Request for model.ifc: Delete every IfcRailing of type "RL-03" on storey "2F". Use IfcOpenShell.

First a look at what the model holds.

```python
import ifcopenshell
import ifcopenshell.util.element

model = ifcopenshell.open("model.ifc")
print(model.schema)
storey = next(s for s in model.by_type("IfcBuildingStorey") if s.Name == "2F")
railings = [e for e in ifcopenshell.util.element.get_decomposition(storey) if e.is_a("IfcRailing")]
seen = {}
for e in railings:
    element_type = ifcopenshell.util.element.get_type(e)
    name = element_type.Name if element_type not in (None, e) else None
    seen[name] = seen.get(name, 0) + 1
for name, count in sorted(seen.items(), key=str):
    print(count, "x", name)
```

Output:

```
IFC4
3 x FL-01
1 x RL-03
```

```python
import ifcopenshell
import ifcopenshell.api.root
import ifcopenshell.util.element

model = ifcopenshell.open("model.ifc")

storey = next(s for s in model.by_type("IfcBuildingStorey") if s.Name == "2F")
railings = [e for e in ifcopenshell.util.element.get_decomposition(storey) if e.is_a("IfcRailing")]
targets = [e for e in railings if (t := ifcopenshell.util.element.get_type(e)) not in (None, e) and t.Name == "RL-03"]

for e in targets:
    ifcopenshell.api.root.remove_product(model, product=e)
print(len(targets), "removed")

model.write("model_updated.ifc")
```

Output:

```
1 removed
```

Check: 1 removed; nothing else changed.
